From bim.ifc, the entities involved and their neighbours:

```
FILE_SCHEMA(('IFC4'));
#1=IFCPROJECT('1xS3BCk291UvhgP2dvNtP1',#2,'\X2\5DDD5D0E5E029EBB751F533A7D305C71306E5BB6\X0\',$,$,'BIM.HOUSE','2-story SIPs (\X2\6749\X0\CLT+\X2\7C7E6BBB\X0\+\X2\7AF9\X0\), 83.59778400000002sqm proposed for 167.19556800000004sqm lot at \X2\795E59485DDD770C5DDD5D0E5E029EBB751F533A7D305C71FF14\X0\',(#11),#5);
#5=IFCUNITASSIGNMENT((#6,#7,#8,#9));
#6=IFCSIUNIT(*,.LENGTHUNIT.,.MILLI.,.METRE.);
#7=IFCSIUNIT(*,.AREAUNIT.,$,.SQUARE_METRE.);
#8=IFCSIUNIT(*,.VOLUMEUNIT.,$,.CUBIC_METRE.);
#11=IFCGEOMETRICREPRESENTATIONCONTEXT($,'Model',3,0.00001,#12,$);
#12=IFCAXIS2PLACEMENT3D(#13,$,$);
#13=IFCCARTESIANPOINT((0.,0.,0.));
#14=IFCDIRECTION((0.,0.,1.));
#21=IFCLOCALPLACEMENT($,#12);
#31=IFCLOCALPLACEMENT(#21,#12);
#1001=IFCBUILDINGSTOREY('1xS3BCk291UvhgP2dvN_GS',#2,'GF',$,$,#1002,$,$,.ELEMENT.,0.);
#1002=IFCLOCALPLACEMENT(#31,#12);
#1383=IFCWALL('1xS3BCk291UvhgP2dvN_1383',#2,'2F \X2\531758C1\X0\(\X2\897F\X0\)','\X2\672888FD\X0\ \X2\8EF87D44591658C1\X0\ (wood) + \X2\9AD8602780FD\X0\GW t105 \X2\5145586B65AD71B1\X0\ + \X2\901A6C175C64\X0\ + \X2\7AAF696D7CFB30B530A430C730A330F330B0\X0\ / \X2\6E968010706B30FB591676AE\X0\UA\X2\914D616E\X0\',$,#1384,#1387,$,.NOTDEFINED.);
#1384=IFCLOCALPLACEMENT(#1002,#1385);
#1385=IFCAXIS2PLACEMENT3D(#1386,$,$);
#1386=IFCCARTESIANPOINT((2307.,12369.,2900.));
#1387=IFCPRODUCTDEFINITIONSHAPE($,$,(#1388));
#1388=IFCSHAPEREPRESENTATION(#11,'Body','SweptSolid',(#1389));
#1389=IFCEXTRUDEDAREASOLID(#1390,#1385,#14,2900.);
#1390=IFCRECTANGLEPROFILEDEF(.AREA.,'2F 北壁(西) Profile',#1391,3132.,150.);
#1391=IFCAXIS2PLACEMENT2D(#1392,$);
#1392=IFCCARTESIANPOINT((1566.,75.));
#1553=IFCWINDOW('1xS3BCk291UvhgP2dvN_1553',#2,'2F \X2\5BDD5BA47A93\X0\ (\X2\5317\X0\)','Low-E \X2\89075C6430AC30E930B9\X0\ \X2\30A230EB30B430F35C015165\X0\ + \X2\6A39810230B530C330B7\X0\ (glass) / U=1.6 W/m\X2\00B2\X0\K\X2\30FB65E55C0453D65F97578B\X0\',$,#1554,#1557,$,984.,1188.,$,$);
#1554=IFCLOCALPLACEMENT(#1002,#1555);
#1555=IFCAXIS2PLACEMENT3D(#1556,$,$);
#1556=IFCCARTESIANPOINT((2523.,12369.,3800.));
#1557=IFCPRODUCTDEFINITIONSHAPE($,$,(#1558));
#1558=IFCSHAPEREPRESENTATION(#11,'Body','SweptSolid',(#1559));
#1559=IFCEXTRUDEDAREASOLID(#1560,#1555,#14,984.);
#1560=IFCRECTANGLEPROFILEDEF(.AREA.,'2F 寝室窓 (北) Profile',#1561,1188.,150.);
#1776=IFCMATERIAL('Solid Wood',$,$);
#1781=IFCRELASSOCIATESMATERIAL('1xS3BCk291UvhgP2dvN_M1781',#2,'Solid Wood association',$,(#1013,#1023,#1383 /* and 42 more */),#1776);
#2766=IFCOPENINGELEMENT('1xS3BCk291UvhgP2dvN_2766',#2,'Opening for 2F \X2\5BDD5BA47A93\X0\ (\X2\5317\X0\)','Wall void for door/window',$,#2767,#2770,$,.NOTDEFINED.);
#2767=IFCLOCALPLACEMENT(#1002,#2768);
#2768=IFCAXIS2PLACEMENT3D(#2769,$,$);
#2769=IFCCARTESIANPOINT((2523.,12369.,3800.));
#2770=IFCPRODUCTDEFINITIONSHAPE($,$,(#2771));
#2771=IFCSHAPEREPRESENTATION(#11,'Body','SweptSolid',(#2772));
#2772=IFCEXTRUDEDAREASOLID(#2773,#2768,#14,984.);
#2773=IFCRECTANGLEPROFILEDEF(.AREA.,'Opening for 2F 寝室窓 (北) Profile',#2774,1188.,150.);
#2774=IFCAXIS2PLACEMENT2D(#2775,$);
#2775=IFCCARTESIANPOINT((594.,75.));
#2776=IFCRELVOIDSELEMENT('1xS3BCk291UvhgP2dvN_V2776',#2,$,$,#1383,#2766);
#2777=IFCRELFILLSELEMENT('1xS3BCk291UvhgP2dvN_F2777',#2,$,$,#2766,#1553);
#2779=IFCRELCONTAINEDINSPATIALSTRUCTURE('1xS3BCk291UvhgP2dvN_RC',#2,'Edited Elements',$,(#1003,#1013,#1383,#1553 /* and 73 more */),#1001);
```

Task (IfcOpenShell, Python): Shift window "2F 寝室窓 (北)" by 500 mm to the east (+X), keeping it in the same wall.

```python
import ifcopenshell
import ifcopenshell.api.geometry
import ifcopenshell.util.placement

model = ifcopenshell.open("bim.ifc")

window = model.by_id(1553)
opening = window.FillsVoids[0].RelatingOpeningElement
wall = opening.VoidsElements[0].RelatingBuildingElement

wall_matrix = ifcopenshell.util.placement.get_local_placement(wall.ObjectPlacement)
shift = wall_matrix[:3, 0] * 500.0
before = ifcopenshell.util.placement.get_local_placement(window.ObjectPlacement)[:3, 3].copy()

# The window is not placed relative to its opening, so move both.
for product in (opening, window):
    matrix = ifcopenshell.util.placement.get_local_placement(product.ObjectPlacement)
    matrix[:3, 3] += shift
    ifcopenshell.api.geometry.edit_object_placement(model, product=product, matrix=matrix, is_si=False)

after = ifcopenshell.util.placement.get_local_placement(window.ObjectPlacement)[:3, 3]
print("window moved by", (after - before).round(3) + 0.0)

model.write("bim_v2.ifc")
```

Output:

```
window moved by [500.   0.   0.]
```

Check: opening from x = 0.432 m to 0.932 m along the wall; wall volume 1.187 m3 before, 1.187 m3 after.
